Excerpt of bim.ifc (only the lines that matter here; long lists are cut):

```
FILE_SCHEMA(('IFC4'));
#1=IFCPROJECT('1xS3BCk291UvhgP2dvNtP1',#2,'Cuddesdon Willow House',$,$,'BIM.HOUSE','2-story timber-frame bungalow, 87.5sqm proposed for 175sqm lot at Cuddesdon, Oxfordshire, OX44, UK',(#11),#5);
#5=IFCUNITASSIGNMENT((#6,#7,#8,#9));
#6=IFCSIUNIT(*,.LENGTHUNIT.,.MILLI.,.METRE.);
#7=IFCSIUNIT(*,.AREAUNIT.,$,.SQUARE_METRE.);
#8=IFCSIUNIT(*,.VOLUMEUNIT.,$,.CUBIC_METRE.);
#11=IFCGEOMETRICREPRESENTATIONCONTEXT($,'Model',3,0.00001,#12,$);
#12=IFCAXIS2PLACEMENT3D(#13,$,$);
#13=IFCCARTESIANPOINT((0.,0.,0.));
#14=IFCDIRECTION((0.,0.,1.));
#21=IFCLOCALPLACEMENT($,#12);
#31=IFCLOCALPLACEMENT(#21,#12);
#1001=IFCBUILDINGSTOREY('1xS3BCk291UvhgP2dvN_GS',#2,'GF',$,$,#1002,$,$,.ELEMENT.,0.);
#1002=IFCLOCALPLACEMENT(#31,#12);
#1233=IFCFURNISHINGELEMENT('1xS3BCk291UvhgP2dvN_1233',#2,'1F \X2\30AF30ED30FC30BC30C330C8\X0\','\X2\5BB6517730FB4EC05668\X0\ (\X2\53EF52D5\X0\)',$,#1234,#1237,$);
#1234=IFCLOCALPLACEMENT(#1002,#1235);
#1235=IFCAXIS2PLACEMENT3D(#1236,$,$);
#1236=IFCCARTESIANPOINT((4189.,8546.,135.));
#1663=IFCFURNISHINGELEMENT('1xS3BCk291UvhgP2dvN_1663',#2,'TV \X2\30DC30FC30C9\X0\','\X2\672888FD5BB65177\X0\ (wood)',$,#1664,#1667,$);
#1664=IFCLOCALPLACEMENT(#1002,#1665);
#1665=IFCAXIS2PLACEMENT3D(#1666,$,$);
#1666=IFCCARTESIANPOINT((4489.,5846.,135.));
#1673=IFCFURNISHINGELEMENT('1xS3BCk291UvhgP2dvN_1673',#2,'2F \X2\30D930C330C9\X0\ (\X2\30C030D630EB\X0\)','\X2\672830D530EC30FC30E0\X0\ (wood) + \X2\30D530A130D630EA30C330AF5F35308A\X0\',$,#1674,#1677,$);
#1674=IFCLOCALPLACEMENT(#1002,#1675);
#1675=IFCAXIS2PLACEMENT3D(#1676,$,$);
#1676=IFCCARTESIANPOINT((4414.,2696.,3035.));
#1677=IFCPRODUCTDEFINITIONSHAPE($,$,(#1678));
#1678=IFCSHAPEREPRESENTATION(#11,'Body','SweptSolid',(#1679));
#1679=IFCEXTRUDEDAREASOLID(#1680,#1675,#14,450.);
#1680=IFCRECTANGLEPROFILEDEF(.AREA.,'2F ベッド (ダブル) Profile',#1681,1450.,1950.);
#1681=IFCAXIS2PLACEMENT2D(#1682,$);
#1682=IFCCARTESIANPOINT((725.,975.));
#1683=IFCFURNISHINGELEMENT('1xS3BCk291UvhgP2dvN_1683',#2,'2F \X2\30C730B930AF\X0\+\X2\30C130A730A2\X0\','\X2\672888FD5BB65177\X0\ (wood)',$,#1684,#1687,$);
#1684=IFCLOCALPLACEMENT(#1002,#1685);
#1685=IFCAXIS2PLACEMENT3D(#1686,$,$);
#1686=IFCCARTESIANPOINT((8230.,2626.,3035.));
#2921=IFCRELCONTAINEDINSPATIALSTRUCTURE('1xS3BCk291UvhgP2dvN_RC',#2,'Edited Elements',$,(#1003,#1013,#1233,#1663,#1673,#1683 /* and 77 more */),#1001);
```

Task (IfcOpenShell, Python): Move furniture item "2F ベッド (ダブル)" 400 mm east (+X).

```python
import ifcopenshell
import ifcopenshell.api.geometry
import ifcopenshell.util.placement
import ifcopenshell.util.unit

model = ifcopenshell.open("bim.ifc")
unit_scale = ifcopenshell.util.unit.calculate_unit_scale(model)

item = model.by_guid("1xS3BCk291UvhgP2dvN_1673")
matrix = ifcopenshell.util.placement.get_local_placement(item.ObjectPlacement)
matrix[0, 3] += 0.4 / unit_scale
ifcopenshell.api.geometry.edit_object_placement(model, product=item, matrix=matrix, is_si=False)

print(ifcopenshell.util.placement.get_local_placement(item.ObjectPlacement).round(3) + 0.0)

model.write("bim_updated.ifc")
```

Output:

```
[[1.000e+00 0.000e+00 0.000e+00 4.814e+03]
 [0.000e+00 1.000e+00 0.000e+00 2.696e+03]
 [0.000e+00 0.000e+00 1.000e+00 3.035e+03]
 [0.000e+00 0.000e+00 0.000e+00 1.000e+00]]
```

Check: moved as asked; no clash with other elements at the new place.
